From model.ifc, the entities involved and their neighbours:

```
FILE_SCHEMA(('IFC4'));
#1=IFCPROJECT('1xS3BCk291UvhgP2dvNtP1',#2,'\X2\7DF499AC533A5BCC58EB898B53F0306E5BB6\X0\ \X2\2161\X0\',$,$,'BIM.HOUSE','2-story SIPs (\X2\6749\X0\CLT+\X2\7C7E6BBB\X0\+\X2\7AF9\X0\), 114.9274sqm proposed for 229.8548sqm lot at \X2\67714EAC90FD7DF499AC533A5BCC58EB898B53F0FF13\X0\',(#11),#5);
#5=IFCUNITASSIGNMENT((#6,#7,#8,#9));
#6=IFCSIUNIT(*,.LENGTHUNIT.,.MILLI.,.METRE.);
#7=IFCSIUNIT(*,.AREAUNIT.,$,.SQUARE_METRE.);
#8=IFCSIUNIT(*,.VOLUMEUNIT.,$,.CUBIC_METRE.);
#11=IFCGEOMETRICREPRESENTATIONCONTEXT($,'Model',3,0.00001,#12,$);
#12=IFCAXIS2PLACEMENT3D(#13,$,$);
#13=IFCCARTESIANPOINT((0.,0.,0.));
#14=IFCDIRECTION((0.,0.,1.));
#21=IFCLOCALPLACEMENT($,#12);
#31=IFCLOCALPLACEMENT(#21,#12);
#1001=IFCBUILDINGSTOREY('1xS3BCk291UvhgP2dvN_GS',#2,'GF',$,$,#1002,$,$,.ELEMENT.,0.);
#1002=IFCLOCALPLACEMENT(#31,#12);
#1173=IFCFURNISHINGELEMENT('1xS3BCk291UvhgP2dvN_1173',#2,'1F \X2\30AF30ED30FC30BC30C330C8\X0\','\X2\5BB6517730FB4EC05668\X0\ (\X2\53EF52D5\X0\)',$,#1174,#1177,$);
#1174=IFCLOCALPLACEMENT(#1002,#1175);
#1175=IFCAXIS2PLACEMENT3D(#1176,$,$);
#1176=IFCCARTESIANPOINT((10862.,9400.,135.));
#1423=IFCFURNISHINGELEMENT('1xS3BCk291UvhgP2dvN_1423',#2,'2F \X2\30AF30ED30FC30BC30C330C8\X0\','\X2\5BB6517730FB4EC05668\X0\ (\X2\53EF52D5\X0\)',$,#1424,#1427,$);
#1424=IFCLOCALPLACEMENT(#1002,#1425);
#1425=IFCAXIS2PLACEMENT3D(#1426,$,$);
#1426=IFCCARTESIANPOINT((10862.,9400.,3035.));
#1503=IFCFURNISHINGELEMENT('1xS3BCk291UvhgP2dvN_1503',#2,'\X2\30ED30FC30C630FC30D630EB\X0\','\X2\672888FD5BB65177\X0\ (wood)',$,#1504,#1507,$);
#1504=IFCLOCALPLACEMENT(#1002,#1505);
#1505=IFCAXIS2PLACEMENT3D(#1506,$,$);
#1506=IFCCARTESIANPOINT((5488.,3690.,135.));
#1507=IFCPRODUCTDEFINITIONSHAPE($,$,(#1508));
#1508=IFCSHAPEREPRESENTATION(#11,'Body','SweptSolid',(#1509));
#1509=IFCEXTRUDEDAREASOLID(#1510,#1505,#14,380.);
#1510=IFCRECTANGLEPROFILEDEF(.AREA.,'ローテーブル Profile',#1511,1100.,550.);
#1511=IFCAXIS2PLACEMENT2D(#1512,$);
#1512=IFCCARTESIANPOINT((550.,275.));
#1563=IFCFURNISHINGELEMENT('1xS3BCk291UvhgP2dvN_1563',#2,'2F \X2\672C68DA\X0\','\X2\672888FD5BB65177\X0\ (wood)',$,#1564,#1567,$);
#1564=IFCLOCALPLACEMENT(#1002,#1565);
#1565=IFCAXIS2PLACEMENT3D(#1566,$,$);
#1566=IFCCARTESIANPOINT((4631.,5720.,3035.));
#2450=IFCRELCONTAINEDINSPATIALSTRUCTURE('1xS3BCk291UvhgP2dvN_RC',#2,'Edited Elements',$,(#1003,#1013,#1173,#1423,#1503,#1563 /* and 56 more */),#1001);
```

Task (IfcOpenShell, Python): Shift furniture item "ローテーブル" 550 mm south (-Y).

```python
import ifcopenshell
import ifcopenshell.api.geometry
import ifcopenshell.util.placement
import ifcopenshell.util.unit

model = ifcopenshell.open("model.ifc")
unit_scale = ifcopenshell.util.unit.calculate_unit_scale(model)

item = model.by_guid("1xS3BCk291UvhgP2dvN_1503")
matrix = ifcopenshell.util.placement.get_local_placement(item.ObjectPlacement)
matrix[1, 3] -= 0.55 / unit_scale
ifcopenshell.api.geometry.edit_object_placement(model, product=item, matrix=matrix, is_si=False)

print(ifcopenshell.util.placement.get_local_placement(item.ObjectPlacement).round(3) + 0.0)

model.write("model_rev.ifc")
```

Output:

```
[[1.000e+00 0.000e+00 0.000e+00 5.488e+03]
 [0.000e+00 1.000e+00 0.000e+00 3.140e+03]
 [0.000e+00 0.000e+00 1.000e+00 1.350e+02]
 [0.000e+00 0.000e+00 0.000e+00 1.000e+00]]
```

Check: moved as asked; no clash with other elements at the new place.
